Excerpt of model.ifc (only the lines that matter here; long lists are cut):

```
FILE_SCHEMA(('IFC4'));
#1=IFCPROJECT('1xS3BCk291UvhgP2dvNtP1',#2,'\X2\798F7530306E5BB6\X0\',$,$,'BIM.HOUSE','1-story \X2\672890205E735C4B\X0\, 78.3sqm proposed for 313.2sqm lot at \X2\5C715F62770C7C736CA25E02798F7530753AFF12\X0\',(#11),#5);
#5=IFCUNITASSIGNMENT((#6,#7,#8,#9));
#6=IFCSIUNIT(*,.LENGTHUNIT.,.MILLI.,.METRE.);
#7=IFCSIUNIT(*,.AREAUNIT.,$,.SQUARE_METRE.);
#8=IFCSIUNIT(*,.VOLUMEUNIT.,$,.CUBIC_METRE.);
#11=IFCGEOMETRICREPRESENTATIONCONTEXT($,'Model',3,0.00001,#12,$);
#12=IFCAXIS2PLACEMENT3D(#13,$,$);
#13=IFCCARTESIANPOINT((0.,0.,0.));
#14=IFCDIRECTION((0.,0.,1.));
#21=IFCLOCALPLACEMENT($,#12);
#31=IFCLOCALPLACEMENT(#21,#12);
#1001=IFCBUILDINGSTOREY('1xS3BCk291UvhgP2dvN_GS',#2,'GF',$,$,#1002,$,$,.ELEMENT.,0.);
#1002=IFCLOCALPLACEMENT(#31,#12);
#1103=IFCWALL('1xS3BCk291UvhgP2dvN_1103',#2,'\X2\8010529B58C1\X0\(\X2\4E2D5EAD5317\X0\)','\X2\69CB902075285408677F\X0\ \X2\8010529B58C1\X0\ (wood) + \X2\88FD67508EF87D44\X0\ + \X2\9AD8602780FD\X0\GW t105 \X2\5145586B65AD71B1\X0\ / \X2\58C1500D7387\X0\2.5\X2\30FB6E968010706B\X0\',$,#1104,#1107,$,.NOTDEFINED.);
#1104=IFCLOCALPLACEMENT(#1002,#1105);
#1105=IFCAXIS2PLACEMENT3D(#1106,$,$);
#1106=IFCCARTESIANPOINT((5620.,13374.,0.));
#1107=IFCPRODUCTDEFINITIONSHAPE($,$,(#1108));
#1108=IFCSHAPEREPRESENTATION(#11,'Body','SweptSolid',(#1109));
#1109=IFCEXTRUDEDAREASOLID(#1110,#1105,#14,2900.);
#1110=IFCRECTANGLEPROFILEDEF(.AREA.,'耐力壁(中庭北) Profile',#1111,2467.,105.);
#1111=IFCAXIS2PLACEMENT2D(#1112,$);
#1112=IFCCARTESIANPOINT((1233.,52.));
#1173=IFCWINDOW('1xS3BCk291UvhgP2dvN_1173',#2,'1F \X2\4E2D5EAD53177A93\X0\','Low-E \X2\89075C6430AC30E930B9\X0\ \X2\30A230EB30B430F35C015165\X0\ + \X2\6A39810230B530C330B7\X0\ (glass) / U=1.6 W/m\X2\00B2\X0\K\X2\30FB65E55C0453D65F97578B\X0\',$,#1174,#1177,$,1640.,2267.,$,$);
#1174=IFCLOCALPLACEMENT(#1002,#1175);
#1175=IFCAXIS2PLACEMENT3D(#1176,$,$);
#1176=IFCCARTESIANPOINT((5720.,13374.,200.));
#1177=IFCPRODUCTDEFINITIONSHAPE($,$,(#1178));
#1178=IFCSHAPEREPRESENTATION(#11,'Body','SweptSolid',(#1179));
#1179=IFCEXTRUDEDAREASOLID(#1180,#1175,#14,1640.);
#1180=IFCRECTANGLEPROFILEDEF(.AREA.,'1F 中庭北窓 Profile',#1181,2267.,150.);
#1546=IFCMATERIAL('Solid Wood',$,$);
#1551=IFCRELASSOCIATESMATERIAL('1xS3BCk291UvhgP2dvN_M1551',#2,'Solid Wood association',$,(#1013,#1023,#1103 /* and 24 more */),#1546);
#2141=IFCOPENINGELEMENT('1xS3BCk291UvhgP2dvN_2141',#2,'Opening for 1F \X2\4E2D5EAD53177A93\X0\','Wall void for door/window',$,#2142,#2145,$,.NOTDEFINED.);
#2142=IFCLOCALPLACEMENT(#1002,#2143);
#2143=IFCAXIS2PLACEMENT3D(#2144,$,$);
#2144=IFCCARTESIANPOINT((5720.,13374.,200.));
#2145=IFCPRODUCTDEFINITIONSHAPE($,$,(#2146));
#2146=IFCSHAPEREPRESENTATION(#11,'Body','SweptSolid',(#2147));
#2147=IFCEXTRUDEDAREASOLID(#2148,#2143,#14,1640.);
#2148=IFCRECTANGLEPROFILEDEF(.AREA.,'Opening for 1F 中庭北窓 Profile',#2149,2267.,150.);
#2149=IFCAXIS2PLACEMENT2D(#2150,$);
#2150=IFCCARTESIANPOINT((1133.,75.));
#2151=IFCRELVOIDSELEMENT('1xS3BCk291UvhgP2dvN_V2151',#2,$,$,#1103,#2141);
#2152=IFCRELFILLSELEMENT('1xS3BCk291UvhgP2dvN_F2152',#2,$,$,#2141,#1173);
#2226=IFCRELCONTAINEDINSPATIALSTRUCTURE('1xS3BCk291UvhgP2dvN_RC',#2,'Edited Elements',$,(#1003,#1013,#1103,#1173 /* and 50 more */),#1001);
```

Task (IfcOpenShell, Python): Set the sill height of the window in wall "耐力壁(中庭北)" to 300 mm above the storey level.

```python
import numpy as np
import ifcopenshell
import ifcopenshell.api.geometry
import ifcopenshell.geom
import ifcopenshell.util.element
import ifcopenshell.util.placement
import ifcopenshell.util.shape
import ifcopenshell.util.unit

model = ifcopenshell.open("model.ifc")
unit_scale = ifcopenshell.util.unit.calculate_unit_scale(model)

window = model.by_guid("1xS3BCk291UvhgP2dvN_1173")
opening = window.FillsVoids[0].RelatingOpeningElement
storey = ifcopenshell.util.element.get_container(window, ifc_class="IfcBuildingStorey")
level = ifcopenshell.util.placement.get_local_placement(storey.ObjectPlacement)[2, 3]

# The opening's origin need not be at the sill, so measure its lowest point.
shape = ifcopenshell.geom.create_shape(ifcopenshell.geom.settings(), opening)
bottom = ifcopenshell.util.shape.get_shape_bottom_elevation(shape, shape.geometry) / unit_scale
dz = level + 0.3 / unit_scale - bottom

shift = np.array([0.0, 0.0, dz])
# The window is not placed relative to its opening, so move both.
for product in (opening, window):
    matrix = ifcopenshell.util.placement.get_local_placement(product.ObjectPlacement)
    matrix[:3, 3] += shift
    ifcopenshell.api.geometry.edit_object_placement(model, product=product, matrix=matrix, is_si=False)

print(f"moved by {dz * unit_scale:+.3f} m")

model.write("model-out.ifc")
```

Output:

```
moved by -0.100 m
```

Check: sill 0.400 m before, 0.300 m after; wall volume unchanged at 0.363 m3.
